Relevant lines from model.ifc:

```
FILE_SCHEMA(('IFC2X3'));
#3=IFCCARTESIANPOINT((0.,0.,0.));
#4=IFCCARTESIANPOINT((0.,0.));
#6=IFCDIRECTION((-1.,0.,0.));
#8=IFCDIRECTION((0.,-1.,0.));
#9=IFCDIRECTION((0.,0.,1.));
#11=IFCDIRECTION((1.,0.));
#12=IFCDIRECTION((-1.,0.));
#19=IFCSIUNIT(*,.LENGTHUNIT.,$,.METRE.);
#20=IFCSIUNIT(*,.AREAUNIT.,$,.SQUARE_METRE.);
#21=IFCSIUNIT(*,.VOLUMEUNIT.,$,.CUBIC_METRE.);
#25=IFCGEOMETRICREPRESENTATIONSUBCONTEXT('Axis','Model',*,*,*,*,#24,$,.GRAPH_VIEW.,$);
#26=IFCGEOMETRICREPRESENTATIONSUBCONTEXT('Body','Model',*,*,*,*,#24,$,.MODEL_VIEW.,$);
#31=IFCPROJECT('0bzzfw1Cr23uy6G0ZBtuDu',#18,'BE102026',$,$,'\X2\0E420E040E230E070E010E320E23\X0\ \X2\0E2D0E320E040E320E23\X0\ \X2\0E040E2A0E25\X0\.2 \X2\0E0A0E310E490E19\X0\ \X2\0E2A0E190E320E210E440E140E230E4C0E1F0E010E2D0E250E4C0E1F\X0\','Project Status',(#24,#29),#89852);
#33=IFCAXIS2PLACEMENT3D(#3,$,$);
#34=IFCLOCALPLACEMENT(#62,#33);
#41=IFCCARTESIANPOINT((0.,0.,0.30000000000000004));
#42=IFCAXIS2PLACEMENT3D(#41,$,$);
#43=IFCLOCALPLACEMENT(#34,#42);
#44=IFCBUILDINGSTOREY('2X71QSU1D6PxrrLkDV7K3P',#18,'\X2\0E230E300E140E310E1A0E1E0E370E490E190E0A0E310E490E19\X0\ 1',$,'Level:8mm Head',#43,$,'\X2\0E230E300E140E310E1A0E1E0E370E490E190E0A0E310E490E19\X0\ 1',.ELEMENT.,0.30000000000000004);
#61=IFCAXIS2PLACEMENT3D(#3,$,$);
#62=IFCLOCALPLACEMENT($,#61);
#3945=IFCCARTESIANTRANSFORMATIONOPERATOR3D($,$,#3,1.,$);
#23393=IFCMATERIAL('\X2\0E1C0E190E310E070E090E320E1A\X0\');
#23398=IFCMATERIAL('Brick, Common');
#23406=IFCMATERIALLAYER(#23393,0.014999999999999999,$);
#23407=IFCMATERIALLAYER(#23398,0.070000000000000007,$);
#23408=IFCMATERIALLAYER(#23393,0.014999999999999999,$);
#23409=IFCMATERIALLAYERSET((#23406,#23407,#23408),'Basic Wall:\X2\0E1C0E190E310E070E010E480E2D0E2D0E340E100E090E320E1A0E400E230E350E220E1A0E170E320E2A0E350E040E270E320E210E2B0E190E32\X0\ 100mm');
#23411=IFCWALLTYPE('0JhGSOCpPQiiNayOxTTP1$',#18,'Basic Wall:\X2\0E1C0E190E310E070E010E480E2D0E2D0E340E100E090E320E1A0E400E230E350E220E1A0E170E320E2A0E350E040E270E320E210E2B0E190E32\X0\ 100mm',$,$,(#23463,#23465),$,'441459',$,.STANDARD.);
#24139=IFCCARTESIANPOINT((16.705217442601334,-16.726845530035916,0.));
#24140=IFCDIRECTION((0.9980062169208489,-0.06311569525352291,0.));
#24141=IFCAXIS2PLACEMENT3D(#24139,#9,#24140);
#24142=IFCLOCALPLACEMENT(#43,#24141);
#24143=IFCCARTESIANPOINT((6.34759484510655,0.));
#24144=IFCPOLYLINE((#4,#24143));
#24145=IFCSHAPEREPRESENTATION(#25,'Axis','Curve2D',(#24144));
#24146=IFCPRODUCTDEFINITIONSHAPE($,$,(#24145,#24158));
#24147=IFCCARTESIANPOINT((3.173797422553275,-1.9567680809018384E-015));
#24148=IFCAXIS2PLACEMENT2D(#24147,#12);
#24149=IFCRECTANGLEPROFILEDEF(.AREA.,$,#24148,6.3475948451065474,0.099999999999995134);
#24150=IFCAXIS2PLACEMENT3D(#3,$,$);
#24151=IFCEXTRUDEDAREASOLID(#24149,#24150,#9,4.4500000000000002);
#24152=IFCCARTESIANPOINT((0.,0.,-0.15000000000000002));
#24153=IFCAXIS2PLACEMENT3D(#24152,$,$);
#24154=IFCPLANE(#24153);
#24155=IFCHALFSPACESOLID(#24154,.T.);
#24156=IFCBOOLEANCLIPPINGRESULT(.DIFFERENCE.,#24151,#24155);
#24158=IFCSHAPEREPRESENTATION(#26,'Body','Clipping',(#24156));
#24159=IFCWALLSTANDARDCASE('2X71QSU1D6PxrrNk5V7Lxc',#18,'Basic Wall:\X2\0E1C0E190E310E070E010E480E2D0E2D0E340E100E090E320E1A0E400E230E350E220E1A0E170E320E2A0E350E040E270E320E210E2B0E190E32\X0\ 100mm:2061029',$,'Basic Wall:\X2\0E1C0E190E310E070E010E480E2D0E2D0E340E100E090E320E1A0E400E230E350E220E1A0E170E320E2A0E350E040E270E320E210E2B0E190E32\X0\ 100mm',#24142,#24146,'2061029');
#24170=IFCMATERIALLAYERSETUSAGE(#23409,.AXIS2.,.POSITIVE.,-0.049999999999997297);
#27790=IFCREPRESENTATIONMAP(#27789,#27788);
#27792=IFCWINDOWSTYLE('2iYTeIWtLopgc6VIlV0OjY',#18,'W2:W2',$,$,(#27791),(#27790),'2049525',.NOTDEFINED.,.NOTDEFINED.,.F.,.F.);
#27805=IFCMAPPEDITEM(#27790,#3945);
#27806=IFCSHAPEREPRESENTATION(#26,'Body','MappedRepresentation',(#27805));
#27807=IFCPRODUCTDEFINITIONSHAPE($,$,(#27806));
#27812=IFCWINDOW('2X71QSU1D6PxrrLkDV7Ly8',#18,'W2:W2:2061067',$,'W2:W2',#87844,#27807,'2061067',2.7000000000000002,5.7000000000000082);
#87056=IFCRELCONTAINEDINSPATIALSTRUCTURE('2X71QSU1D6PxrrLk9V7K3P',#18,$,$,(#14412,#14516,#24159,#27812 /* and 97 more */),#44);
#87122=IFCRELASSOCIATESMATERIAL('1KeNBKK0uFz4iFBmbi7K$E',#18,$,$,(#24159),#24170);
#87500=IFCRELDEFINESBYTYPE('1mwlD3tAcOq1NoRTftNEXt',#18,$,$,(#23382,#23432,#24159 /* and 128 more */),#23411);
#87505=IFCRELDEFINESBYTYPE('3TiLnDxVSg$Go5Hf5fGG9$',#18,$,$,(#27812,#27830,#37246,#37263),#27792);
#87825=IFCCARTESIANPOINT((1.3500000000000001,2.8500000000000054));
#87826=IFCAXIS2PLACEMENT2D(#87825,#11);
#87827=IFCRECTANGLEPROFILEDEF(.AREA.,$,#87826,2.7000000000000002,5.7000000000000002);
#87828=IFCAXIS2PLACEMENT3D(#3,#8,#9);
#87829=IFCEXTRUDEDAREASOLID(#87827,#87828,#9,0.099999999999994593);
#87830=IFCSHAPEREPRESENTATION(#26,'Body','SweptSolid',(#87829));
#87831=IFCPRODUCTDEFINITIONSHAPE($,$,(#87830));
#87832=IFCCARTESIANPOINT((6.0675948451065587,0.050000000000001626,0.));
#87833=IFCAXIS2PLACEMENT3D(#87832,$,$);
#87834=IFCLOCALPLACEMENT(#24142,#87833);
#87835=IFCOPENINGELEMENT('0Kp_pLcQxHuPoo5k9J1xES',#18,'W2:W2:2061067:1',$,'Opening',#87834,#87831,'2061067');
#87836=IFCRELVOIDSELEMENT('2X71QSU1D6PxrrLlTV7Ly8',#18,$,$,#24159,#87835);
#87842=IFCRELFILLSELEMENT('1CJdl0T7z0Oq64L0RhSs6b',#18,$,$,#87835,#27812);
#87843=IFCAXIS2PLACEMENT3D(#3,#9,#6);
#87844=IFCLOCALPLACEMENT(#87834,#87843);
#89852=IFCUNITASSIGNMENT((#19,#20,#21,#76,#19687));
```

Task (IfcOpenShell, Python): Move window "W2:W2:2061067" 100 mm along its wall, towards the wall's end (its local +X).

```python
import ifcopenshell
import ifcopenshell.api.geometry
import ifcopenshell.util.placement

model = ifcopenshell.open("model.ifc")

window = model.by_guid("2X71QSU1D6PxrrLkDV7Ly8")
opening = window.FillsVoids[0].RelatingOpeningElement
wall = opening.VoidsElements[0].RelatingBuildingElement

wall_matrix = ifcopenshell.util.placement.get_local_placement(wall.ObjectPlacement)
shift = wall_matrix[:3, 0] * 0.1
before = ifcopenshell.util.placement.get_local_placement(window.ObjectPlacement)[:3, 3].copy()

# The window is placed relative to its opening, so it follows when the opening moves.
matrix = ifcopenshell.util.placement.get_local_placement(opening.ObjectPlacement)
matrix[:3, 3] += shift
ifcopenshell.api.geometry.edit_object_placement(
    model, product=opening, matrix=matrix, is_si=False, should_transform_children=True
)

after = ifcopenshell.util.placement.get_local_placement(window.ObjectPlacement)[:3, 3]
print("window moved by", (after - before).round(3) + 0.0)

model.write("model_updated.ifc")
```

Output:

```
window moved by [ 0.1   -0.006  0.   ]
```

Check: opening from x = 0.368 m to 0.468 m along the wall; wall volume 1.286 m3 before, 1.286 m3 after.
